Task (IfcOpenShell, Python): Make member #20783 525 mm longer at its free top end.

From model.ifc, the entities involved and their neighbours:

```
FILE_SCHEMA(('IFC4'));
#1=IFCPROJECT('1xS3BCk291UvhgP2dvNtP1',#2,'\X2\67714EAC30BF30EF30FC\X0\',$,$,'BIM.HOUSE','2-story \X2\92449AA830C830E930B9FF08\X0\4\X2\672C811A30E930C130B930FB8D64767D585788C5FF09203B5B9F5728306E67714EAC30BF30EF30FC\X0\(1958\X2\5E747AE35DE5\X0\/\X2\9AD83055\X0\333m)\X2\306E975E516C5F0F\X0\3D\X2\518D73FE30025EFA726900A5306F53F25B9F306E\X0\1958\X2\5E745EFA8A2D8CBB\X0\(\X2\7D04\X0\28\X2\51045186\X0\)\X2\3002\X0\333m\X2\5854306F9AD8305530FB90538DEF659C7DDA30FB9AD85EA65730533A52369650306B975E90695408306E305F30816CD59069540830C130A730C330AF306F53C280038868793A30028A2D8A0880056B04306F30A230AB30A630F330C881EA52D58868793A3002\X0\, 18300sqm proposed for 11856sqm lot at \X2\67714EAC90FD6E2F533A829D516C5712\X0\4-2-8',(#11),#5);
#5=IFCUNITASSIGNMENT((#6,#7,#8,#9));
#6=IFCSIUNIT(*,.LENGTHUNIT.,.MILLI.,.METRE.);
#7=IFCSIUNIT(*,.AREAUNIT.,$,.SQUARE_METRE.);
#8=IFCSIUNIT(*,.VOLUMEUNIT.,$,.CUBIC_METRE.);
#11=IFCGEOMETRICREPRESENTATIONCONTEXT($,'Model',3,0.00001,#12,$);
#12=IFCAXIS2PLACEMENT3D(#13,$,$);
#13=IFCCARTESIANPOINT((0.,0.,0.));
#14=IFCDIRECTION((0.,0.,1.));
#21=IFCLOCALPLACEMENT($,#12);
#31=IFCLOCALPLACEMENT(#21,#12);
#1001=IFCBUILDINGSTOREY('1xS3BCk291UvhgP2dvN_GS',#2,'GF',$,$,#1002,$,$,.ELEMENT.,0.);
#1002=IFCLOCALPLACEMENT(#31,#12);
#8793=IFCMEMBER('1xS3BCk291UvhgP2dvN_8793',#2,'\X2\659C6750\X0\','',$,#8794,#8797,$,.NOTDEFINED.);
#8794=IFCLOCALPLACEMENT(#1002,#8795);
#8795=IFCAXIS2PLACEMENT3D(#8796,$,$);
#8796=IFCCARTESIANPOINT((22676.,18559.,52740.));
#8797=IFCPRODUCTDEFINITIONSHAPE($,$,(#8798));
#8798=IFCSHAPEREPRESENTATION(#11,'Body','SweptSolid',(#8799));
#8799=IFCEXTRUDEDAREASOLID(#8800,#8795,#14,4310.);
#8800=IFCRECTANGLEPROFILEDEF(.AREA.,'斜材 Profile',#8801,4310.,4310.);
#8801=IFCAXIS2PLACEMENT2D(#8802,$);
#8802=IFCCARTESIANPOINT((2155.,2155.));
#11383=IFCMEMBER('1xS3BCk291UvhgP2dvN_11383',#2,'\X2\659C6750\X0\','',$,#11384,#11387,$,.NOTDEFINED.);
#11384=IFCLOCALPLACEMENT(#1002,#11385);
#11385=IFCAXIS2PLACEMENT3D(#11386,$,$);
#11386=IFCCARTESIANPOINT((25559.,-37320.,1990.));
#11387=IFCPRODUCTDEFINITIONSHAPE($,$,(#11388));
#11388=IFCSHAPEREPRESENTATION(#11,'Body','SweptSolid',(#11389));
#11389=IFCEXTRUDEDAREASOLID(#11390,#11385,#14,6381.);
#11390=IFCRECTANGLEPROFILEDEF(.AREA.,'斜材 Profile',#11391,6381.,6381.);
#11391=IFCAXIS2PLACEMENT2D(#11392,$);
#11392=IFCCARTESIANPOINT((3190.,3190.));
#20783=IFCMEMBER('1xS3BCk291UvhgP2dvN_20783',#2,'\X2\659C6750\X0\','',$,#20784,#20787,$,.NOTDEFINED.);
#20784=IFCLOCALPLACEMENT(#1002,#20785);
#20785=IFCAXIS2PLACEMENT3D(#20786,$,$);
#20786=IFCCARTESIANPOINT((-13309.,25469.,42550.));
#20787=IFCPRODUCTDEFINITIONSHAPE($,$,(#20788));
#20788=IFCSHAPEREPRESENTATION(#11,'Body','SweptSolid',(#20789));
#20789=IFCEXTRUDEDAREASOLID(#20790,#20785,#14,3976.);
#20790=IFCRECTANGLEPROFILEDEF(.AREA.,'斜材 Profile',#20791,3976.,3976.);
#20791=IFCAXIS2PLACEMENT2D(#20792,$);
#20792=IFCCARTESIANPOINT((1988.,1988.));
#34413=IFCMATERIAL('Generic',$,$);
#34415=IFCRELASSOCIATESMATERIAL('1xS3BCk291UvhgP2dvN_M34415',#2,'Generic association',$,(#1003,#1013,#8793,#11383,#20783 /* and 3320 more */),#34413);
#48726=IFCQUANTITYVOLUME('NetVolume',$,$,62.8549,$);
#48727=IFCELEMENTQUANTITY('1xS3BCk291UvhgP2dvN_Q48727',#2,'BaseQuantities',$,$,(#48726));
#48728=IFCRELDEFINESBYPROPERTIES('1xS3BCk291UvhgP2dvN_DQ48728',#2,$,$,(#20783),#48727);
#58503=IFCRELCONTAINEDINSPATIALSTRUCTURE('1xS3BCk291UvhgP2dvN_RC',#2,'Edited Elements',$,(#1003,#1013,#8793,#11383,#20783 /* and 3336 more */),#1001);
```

```python
import ifcopenshell
import ifcopenshell.api.pset
import ifcopenshell.util.element
import ifcopenshell.util.unit

model = ifcopenshell.open("model.ifc")
unit_scale = ifcopenshell.util.unit.calculate_unit_scale(model)

member = model.by_guid("1xS3BCk291UvhgP2dvN_20783")
change = 0.525 / unit_scale

# The extrusion runs towards the end named, so only its depth changes.
body = next(r for r in member.Representation.Representations if r.RepresentationIdentifier == "Body")
solid = body.Items[0]
old_length = solid.Depth
solid.Depth += change

# Update the stored length and volume.
qto = model.by_id(ifcopenshell.util.element.get_pset(member, "BaseQuantities", should_inherit=False)["id"])
ifcopenshell.api.pset.edit_qto(model, qto=qto, properties={
    "NetVolume": ifcopenshell.util.element.get_pset(member, "BaseQuantities", "NetVolume") * solid.Depth / old_length,
})

print(f"length {old_length:g} -> {solid.Depth:g}")

model.write("model_rev.ifc")
```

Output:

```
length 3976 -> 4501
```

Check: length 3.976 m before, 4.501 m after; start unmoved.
